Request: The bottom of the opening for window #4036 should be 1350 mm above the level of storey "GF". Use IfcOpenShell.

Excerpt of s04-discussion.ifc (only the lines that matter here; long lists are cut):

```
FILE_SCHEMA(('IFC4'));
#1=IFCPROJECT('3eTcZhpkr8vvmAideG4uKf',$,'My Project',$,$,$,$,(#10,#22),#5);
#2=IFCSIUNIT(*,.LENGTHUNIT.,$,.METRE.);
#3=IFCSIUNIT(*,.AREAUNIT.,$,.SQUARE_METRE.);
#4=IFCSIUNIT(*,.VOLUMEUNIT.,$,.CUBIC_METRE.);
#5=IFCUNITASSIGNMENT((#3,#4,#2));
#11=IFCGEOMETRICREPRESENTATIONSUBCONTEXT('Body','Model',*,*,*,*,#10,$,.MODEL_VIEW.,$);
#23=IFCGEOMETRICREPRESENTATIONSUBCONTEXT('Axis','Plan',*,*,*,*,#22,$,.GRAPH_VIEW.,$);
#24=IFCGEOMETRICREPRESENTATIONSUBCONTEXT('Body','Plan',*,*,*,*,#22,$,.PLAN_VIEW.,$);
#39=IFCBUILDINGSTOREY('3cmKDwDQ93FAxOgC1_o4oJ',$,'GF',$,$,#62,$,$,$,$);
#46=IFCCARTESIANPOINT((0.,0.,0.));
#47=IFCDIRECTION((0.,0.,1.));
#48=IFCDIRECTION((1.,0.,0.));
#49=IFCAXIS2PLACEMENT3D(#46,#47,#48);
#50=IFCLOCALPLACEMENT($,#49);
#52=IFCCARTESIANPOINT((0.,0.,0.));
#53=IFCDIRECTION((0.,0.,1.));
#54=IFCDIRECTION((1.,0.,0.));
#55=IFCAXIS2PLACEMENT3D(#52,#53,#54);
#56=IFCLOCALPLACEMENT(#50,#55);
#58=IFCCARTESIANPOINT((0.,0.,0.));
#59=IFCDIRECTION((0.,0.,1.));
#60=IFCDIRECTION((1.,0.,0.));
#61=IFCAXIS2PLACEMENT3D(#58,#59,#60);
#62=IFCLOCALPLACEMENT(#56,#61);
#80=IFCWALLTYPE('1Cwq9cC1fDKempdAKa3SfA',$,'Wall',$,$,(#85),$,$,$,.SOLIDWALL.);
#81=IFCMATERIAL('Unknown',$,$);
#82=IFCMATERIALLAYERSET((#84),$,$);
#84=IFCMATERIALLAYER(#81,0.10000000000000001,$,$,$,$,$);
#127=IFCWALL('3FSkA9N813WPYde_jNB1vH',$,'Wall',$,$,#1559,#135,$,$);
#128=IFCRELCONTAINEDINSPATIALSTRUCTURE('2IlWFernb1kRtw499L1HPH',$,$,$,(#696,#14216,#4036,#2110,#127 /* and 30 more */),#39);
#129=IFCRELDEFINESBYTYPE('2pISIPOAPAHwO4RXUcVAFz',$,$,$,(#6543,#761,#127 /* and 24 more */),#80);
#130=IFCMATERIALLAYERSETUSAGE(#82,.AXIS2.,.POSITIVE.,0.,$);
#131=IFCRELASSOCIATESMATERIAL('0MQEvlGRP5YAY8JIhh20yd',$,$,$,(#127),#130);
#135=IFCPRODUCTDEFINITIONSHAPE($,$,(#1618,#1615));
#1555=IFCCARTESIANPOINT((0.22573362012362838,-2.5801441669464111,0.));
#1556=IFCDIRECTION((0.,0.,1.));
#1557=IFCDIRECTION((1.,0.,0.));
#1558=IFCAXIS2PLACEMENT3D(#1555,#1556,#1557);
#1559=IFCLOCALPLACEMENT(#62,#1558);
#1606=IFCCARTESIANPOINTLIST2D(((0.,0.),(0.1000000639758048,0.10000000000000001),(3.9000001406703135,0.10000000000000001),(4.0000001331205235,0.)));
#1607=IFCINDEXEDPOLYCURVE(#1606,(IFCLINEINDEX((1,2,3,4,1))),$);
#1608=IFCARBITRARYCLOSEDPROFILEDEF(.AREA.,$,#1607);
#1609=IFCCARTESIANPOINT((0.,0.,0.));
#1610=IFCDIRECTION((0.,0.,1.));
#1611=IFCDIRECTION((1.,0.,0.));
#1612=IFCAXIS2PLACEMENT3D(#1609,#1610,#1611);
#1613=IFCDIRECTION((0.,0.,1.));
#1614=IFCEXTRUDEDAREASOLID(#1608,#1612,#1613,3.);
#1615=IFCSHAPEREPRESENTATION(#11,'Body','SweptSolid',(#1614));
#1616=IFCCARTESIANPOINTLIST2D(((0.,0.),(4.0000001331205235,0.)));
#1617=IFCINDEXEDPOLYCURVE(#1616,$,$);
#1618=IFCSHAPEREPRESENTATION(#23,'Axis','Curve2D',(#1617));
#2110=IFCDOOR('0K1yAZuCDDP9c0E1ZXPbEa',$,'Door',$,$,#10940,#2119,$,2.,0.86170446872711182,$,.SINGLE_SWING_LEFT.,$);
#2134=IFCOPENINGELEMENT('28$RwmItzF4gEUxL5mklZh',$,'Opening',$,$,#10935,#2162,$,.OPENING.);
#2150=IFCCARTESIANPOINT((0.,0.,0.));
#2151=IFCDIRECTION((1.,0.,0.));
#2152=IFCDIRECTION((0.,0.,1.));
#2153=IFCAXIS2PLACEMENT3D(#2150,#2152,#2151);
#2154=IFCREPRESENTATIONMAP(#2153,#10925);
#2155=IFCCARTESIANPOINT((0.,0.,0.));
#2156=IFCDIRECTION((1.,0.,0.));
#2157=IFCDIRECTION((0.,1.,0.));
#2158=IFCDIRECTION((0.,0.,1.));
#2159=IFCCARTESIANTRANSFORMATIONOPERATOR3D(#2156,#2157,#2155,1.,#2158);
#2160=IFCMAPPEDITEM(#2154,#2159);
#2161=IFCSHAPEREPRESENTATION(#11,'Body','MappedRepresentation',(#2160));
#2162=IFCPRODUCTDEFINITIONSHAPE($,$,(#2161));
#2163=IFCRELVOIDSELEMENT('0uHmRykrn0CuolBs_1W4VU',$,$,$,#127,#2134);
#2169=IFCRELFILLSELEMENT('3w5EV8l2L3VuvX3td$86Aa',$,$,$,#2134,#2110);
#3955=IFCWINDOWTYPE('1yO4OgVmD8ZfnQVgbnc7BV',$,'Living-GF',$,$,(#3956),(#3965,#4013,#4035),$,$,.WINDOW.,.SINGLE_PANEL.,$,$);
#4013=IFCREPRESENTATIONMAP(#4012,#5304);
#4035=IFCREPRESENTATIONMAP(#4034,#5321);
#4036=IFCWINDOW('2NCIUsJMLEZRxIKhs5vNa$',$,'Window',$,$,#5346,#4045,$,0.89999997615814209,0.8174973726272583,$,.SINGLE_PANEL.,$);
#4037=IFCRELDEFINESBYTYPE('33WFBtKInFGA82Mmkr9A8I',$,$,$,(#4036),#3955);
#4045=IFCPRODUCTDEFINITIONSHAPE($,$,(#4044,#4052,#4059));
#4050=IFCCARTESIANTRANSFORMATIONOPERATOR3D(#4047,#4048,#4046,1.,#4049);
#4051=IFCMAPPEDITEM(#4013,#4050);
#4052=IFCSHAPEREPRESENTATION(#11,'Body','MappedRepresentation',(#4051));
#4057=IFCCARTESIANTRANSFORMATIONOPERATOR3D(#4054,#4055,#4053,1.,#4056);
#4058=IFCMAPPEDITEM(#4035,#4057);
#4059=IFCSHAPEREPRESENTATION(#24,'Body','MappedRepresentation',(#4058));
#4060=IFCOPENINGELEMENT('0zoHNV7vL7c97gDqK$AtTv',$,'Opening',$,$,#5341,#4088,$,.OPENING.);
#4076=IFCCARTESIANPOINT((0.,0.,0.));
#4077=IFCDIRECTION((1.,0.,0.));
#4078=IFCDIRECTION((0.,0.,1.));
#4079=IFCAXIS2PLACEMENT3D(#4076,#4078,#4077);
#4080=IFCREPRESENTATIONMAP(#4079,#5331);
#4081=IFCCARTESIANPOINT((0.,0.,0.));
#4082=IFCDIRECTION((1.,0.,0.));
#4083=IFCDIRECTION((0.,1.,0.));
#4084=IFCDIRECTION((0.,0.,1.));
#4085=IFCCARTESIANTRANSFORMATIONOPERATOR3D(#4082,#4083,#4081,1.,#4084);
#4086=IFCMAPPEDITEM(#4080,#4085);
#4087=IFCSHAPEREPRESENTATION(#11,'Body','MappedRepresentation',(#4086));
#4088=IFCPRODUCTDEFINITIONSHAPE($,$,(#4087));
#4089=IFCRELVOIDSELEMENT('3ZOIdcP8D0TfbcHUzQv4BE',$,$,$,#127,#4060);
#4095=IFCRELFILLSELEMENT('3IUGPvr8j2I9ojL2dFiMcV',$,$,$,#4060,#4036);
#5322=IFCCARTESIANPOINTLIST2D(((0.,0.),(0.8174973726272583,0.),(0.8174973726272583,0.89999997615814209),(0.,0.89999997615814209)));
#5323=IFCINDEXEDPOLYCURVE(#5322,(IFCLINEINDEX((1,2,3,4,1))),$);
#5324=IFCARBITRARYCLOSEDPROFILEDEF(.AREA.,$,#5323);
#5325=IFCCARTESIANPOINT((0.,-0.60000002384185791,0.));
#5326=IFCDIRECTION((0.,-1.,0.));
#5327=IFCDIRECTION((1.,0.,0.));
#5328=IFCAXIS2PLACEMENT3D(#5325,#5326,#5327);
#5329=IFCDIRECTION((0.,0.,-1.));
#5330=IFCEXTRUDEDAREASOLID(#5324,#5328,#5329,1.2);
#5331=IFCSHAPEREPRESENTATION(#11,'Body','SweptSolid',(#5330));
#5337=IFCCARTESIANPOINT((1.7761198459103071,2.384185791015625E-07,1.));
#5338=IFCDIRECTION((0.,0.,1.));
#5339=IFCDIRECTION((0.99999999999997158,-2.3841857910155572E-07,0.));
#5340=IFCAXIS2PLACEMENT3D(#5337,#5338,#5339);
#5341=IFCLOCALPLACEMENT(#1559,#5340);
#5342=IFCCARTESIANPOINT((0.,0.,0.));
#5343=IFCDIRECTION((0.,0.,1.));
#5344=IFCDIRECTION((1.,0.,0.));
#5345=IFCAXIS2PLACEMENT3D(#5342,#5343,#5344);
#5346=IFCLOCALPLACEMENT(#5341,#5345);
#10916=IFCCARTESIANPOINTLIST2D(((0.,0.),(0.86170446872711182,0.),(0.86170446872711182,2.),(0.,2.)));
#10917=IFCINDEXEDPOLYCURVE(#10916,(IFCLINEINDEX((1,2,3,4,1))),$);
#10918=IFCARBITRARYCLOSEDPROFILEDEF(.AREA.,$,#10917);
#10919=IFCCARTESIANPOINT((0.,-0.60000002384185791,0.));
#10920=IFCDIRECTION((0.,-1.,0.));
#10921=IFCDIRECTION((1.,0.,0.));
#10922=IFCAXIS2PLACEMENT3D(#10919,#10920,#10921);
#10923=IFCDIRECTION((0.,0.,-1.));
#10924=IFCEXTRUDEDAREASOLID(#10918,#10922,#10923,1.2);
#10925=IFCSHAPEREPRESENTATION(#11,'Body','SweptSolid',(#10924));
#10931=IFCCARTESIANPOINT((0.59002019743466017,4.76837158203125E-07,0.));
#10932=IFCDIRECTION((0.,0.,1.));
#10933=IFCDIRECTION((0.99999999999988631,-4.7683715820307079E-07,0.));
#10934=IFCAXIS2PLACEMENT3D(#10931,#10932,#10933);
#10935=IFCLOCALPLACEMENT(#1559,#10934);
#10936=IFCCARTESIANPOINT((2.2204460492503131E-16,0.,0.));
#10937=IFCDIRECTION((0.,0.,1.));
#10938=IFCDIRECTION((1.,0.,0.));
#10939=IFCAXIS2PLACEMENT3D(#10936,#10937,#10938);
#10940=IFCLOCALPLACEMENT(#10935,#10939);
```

```python
import numpy as np
import ifcopenshell
import ifcopenshell.api.geometry
import ifcopenshell.geom
import ifcopenshell.util.element
import ifcopenshell.util.placement
import ifcopenshell.util.shape
import ifcopenshell.util.unit

model = ifcopenshell.open("s04-discussion.ifc")
unit_scale = ifcopenshell.util.unit.calculate_unit_scale(model)

window = model.by_id(4036)
opening = window.FillsVoids[0].RelatingOpeningElement
storey = ifcopenshell.util.element.get_container(window, ifc_class="IfcBuildingStorey")
level = ifcopenshell.util.placement.get_local_placement(storey.ObjectPlacement)[2, 3]

# The opening's origin need not be at the sill, so measure its lowest point.
shape = ifcopenshell.geom.create_shape(ifcopenshell.geom.settings(), opening)
bottom = ifcopenshell.util.shape.get_shape_bottom_elevation(shape, shape.geometry) / unit_scale
dz = level + 1.35 / unit_scale - bottom

shift = np.array([0.0, 0.0, dz])
# The window is placed relative to its opening, so it follows when the opening moves.
matrix = ifcopenshell.util.placement.get_local_placement(opening.ObjectPlacement)
matrix[:3, 3] += shift
ifcopenshell.api.geometry.edit_object_placement(
    model, product=opening, matrix=matrix, is_si=False, should_transform_children=True
)

print(f"moved by {dz * unit_scale:+.3f} m")

model.write("s04-discussion_rev.ifc")
```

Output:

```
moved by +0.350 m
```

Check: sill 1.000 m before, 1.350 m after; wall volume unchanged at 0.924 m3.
